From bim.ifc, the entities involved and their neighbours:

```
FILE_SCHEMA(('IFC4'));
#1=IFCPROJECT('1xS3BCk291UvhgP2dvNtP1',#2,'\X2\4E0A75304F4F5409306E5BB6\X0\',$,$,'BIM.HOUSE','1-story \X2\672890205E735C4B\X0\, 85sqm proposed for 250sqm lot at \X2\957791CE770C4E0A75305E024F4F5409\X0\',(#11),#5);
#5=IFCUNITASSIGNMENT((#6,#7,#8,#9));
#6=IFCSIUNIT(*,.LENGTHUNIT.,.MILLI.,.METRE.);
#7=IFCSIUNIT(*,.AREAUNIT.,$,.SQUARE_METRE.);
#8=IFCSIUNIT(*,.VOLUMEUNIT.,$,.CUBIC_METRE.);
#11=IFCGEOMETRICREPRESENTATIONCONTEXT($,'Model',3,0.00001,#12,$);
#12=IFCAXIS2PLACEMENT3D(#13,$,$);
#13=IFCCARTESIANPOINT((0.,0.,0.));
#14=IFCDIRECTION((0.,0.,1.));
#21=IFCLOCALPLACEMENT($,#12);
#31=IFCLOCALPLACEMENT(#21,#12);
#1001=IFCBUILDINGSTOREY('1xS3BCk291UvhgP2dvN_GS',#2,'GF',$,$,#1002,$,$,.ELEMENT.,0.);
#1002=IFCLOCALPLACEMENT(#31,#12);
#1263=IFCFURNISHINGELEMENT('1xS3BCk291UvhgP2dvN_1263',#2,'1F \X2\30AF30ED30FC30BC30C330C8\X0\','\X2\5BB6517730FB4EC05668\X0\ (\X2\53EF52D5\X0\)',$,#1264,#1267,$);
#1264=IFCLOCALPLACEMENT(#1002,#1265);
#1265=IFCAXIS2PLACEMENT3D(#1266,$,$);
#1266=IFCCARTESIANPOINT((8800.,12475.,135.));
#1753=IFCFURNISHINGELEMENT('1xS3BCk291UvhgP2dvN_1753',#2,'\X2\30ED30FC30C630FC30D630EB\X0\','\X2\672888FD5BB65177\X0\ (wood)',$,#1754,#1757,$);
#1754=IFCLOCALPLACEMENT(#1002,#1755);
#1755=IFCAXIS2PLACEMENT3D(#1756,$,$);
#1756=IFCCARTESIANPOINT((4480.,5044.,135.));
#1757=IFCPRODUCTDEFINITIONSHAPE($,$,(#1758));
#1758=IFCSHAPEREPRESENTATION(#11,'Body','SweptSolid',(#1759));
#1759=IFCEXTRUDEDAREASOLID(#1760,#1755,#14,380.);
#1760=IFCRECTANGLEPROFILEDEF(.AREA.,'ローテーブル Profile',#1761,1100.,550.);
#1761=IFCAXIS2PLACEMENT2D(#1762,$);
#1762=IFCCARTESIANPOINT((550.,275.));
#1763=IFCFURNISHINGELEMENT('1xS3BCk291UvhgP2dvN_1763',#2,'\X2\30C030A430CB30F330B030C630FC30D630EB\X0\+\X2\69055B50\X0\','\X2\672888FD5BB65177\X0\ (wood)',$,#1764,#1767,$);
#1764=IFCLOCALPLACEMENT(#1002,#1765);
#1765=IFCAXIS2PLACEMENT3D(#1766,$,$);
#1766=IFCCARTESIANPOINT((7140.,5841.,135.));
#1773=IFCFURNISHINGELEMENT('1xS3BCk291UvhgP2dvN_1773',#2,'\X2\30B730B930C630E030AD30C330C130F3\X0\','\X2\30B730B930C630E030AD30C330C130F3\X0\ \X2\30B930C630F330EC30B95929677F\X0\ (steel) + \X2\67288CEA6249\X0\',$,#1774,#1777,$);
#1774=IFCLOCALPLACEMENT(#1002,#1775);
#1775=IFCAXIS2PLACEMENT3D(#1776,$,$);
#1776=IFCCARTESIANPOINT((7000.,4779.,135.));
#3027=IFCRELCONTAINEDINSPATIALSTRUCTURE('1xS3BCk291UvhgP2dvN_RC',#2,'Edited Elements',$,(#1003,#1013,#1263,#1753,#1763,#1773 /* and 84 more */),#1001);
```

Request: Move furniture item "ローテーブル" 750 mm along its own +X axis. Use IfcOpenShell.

```python
import ifcopenshell
import ifcopenshell.api.geometry
import ifcopenshell.util.placement
import ifcopenshell.util.unit

model = ifcopenshell.open("bim.ifc")
unit_scale = ifcopenshell.util.unit.calculate_unit_scale(model)

item = model.by_guid("1xS3BCk291UvhgP2dvN_1753")
matrix = ifcopenshell.util.placement.get_local_placement(item.ObjectPlacement)
matrix[:3, 3] += matrix[:3, 0] * 0.75 / unit_scale
ifcopenshell.api.geometry.edit_object_placement(model, product=item, matrix=matrix, is_si=False)

print(ifcopenshell.util.placement.get_local_placement(item.ObjectPlacement).round(3) + 0.0)

model.write("bim-out.ifc")
```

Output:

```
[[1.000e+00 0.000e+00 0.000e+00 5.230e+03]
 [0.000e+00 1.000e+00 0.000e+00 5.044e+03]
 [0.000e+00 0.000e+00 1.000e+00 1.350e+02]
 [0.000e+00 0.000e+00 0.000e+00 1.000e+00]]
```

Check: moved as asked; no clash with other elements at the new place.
